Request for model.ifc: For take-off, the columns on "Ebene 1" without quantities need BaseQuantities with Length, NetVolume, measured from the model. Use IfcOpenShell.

First a look at what the model holds.

```python
import ifcopenshell
import ifcopenshell.util.element
import ifcopenshell.util.unit

model = ifcopenshell.open("model.ifc")
print(model.schema)
for unit_type in ("LENGTHUNIT", "AREAUNIT", "VOLUMEUNIT"):
    print(unit_type, ifcopenshell.util.unit.calculate_unit_scale(model, unit_type))
storey = next(s for s in model.by_type("IfcBuildingStorey") if s.Name == "Ebene 1")
columns = [e for e in ifcopenshell.util.element.get_decomposition(storey) if e.is_a("IfcColumn")]
for e in sorted(columns, key=lambda e: e.id()):
    print(e.id(), e.is_a(), e.Name, list(ifcopenshell.util.element.get_psets(e, qtos_only=True)), sep=" | ")
```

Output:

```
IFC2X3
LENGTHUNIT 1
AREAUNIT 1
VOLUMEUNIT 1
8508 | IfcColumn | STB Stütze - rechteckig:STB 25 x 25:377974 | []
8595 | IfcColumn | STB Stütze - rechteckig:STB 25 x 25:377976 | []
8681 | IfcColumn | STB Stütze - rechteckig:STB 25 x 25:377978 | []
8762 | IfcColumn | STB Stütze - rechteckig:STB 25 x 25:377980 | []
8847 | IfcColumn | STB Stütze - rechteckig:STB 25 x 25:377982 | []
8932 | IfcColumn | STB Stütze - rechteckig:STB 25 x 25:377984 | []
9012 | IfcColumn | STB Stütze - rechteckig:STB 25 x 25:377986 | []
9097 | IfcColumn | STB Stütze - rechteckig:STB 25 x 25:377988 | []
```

```python
import ifcopenshell
import ifcopenshell.api.pset
import ifcopenshell.geom
import ifcopenshell.util.element
import ifcopenshell.util.shape
import ifcopenshell.util.unit

model = ifcopenshell.open("model.ifc")
unit_scale = ifcopenshell.util.unit.calculate_unit_scale(model)
volume_scale = ifcopenshell.util.unit.calculate_unit_scale(model, "VOLUMEUNIT")
settings = ifcopenshell.geom.settings()

storey = next(s for s in model.by_type("IfcBuildingStorey") if s.Name == "Ebene 1")
columns = [e for e in ifcopenshell.util.element.get_decomposition(storey) if e.is_a("IfcColumn")]

for e in sorted(columns, key=lambda e: e.id()):
    if ifcopenshell.util.element.get_psets(e, qtos_only=True, should_inherit=False):
        continue
    # Geometry comes back in metres, in the element's own axes.
    shape = ifcopenshell.geom.create_shape(settings, e)
    values = {
        "Length": ifcopenshell.util.shape.get_z(shape.geometry) / unit_scale,
        "NetVolume": ifcopenshell.util.shape.get_volume(shape.geometry) / volume_scale,
    }
    qto = ifcopenshell.api.pset.add_qto(model, product=e, name="BaseQuantities")
    ifcopenshell.api.pset.edit_qto(model, qto=qto, properties=values)
    print(e.id(), {k: round(v, 3) for k, v in values.items()})

model.write("model_edited.ifc")
```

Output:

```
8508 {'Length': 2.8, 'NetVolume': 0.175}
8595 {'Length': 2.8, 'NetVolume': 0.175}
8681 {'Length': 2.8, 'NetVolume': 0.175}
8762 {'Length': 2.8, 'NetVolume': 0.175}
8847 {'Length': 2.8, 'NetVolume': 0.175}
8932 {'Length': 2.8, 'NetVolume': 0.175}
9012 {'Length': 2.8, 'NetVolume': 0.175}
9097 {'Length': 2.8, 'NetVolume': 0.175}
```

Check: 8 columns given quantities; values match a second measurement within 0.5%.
